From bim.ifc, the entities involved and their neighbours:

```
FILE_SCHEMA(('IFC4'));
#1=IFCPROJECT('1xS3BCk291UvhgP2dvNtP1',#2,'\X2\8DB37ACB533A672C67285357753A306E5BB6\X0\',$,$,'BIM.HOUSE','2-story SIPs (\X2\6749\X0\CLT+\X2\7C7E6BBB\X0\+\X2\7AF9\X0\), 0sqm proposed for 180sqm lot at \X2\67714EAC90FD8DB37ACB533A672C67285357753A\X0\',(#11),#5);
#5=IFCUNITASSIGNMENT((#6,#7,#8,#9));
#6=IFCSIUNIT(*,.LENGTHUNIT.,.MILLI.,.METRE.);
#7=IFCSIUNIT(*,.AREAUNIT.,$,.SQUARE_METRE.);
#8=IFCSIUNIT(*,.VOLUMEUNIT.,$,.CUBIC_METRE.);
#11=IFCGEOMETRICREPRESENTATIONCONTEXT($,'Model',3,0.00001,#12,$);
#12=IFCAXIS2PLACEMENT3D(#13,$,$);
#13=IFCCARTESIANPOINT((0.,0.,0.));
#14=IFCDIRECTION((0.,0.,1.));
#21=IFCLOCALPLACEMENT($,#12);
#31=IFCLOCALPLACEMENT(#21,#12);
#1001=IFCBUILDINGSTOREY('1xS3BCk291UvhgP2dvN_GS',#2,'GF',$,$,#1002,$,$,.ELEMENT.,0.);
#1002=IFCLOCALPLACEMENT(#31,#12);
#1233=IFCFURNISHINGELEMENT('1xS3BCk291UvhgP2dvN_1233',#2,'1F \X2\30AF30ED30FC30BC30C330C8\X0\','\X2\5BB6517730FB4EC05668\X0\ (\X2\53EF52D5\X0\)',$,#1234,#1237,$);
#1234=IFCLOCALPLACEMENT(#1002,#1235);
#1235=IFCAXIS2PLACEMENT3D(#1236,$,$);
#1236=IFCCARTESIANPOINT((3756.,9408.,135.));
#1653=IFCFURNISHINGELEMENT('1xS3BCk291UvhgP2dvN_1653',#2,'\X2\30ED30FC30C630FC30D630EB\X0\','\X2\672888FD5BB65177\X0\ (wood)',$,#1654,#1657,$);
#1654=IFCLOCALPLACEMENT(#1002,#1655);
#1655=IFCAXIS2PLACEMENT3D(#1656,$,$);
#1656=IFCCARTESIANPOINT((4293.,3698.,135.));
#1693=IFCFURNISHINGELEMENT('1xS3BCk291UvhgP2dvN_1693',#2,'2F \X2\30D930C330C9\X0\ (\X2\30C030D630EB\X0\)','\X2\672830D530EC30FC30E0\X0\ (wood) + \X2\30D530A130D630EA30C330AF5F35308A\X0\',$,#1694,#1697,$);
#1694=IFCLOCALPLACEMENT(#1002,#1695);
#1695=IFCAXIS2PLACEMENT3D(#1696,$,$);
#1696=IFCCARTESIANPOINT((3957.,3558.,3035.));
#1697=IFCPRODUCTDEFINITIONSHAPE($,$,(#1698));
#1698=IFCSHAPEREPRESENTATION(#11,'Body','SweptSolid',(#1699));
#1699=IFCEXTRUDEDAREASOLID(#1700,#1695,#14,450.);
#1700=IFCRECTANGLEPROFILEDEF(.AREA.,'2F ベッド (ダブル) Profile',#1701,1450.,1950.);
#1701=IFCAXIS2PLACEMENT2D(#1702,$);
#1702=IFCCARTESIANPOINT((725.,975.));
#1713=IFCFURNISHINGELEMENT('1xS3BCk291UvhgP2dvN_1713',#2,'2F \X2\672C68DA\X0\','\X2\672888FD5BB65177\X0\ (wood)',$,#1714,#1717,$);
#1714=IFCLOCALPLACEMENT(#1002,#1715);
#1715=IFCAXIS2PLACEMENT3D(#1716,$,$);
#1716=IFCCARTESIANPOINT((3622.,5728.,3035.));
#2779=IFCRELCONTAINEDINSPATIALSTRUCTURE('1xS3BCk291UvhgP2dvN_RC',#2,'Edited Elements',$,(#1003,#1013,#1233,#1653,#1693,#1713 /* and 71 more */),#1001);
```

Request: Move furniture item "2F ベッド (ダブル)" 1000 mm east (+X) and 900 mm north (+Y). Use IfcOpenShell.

```python
import ifcopenshell
import ifcopenshell.api.geometry
import ifcopenshell.util.placement
import ifcopenshell.util.unit

model = ifcopenshell.open("bim.ifc")
unit_scale = ifcopenshell.util.unit.calculate_unit_scale(model)

item = model.by_guid("1xS3BCk291UvhgP2dvN_1693")
matrix = ifcopenshell.util.placement.get_local_placement(item.ObjectPlacement)
matrix[0, 3] += 1 / unit_scale
matrix[1, 3] += 0.9 / unit_scale
ifcopenshell.api.geometry.edit_object_placement(model, product=item, matrix=matrix, is_si=False)

print(ifcopenshell.util.placement.get_local_placement(item.ObjectPlacement).round(3) + 0.0)

model.write("bim_rev.ifc")
```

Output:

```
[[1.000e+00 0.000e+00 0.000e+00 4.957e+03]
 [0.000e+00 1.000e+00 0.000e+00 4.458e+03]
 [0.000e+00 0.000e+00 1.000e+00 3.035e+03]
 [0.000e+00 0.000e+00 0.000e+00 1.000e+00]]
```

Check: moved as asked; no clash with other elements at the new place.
